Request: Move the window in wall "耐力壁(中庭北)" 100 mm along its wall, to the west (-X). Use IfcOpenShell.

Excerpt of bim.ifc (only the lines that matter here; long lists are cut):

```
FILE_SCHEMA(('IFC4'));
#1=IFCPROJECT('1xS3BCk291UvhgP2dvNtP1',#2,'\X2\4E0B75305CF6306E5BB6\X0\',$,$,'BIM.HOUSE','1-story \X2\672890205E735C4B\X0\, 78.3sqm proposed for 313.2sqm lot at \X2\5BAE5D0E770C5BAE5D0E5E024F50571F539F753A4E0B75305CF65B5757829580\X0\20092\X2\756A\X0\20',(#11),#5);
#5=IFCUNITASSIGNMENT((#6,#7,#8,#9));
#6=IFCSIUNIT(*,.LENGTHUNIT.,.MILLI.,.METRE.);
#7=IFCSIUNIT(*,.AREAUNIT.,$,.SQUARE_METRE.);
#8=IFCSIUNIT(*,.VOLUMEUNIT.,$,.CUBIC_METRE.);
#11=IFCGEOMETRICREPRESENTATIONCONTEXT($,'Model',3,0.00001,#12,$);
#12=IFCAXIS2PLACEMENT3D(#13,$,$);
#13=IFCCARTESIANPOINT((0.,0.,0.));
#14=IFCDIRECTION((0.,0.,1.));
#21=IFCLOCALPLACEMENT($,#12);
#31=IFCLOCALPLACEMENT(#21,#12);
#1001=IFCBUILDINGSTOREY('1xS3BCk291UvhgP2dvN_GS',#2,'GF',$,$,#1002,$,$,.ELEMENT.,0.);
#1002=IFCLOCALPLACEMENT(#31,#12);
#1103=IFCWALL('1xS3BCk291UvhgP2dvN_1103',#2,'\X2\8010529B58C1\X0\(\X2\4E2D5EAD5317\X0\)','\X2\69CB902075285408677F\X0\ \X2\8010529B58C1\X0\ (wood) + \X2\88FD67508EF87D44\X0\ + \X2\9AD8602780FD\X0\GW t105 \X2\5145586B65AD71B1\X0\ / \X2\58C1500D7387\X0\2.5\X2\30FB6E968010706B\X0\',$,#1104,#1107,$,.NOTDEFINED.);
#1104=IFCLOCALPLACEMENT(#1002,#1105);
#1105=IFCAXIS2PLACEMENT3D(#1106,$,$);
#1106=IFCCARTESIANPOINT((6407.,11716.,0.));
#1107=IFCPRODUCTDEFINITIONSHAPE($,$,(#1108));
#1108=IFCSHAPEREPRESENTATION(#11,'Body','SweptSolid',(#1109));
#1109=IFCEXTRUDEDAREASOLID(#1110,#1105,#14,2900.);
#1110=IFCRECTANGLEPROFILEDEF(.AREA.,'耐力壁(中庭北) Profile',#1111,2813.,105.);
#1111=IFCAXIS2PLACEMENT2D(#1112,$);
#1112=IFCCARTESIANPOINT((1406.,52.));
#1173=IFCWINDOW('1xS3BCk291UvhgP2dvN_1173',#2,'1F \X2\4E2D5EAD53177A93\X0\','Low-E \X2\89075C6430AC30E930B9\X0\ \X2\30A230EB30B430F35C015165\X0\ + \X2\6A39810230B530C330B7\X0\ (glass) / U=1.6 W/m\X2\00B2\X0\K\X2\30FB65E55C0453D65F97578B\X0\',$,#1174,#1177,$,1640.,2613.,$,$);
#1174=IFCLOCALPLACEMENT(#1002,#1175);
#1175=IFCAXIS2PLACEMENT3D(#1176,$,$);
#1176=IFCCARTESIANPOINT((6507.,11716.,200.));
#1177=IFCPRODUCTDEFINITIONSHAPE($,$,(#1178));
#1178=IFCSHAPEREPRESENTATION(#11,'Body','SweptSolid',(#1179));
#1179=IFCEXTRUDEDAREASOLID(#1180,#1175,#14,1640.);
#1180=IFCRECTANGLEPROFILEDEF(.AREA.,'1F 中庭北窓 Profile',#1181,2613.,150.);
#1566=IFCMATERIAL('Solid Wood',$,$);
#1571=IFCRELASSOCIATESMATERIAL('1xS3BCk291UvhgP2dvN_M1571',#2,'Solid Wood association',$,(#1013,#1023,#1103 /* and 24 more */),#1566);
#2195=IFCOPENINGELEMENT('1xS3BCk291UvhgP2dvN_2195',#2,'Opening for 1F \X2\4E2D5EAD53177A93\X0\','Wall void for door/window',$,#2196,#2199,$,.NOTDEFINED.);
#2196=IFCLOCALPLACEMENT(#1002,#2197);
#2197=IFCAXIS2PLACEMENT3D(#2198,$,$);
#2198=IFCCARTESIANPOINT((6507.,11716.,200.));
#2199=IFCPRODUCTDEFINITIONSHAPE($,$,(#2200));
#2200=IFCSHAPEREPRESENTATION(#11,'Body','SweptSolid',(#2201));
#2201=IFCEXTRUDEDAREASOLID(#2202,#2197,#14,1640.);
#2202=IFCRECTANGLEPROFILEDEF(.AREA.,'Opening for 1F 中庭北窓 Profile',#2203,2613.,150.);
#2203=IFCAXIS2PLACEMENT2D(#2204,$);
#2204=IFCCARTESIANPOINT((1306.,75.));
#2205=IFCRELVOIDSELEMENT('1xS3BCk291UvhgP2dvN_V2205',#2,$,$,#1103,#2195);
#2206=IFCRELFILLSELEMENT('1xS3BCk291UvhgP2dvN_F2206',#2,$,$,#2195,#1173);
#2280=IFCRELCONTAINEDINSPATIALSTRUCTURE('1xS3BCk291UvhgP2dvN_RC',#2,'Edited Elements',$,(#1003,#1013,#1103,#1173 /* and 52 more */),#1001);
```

```python
import ifcopenshell
import ifcopenshell.api.geometry
import ifcopenshell.util.placement

model = ifcopenshell.open("bim.ifc")

window = model.by_id(1173)
opening = window.FillsVoids[0].RelatingOpeningElement
wall = opening.VoidsElements[0].RelatingBuildingElement

wall_matrix = ifcopenshell.util.placement.get_local_placement(wall.ObjectPlacement)
shift = wall_matrix[:3, 0] * -100.0
before = ifcopenshell.util.placement.get_local_placement(window.ObjectPlacement)[:3, 3].copy()

# The window is not placed relative to its opening, so move both.
for product in (opening, window):
    matrix = ifcopenshell.util.placement.get_local_placement(product.ObjectPlacement)
    matrix[:3, 3] += shift
    ifcopenshell.api.geometry.edit_object_placement(model, product=product, matrix=matrix, is_si=False)

after = ifcopenshell.util.placement.get_local_placement(window.ObjectPlacement)[:3, 3]
print("window moved by", (after - before).round(3) + 0.0)

model.write("bim_edited.ifc")
```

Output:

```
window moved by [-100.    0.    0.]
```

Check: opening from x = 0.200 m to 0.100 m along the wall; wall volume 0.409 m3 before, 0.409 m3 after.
